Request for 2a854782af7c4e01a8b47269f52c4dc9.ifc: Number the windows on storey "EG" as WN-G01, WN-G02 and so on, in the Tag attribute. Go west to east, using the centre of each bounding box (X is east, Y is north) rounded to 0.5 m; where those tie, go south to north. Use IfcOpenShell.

First a look at what the model holds.

```python
import ifcopenshell
import ifcopenshell.util.element
import ifcopenshell.util.placement

model = ifcopenshell.open("2a854782af7c4e01a8b47269f52c4dc9.ifc")
print(model.schema)
storey = next(s for s in model.by_type("IfcBuildingStorey") if s.Name == "EG")
windows = [e for e in ifcopenshell.util.element.get_decomposition(storey) if e.is_a("IfcWindow")]
for e in sorted(windows, key=lambda e: e.id()):
    origin = ifcopenshell.util.placement.get_local_placement(e.ObjectPlacement)[:3, 3]
    print(e.id(), e.Tag, e.Name, origin.round(2) + 0.0, sep=" | ")
```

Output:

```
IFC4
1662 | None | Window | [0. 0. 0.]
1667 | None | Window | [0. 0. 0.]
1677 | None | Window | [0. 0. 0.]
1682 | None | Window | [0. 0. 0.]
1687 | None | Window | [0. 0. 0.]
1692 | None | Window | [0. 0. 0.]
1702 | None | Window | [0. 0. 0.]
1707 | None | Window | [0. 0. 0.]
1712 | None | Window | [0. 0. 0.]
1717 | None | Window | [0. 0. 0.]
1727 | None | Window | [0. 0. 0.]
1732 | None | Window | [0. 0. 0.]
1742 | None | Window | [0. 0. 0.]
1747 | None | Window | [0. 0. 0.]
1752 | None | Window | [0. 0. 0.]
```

```python
import ifcopenshell
import ifcopenshell.geom
import ifcopenshell.util.element
import ifcopenshell.util.shape

model = ifcopenshell.open("2a854782af7c4e01a8b47269f52c4dc9.ifc")
settings = ifcopenshell.geom.settings()
settings.set("use-world-coords", True)


def centre(element):
    shape = ifcopenshell.geom.create_shape(settings, element)
    return ifcopenshell.util.shape.get_bbox_centroid(shape.geometry)


storey = next(s for s in model.by_type("IfcBuildingStorey") if s.Name == "EG")
windows = [e for e in ifcopenshell.util.element.get_decomposition(storey) if e.is_a("IfcWindow")]

# Insertion points can sit at a corner or the storey origin, so sort by the geometry (in metres).
centres = {e: centre(e) for e in windows}
windows.sort(key=lambda e: (round(centres[e][0] / 0.5), centres[e][1]))

for i, e in enumerate(windows, start=1):
    number = f"WN-G{i:02d}"
    e.Tag = number
    print(e.id(), number)

model.write("2a854782af7c4e01a8b47269f52c4dc9_v2.ifc")
```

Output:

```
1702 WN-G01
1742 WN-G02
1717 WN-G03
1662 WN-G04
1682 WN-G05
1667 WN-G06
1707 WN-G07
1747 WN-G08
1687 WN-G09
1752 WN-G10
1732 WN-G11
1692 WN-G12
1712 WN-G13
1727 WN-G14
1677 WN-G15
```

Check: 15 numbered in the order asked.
